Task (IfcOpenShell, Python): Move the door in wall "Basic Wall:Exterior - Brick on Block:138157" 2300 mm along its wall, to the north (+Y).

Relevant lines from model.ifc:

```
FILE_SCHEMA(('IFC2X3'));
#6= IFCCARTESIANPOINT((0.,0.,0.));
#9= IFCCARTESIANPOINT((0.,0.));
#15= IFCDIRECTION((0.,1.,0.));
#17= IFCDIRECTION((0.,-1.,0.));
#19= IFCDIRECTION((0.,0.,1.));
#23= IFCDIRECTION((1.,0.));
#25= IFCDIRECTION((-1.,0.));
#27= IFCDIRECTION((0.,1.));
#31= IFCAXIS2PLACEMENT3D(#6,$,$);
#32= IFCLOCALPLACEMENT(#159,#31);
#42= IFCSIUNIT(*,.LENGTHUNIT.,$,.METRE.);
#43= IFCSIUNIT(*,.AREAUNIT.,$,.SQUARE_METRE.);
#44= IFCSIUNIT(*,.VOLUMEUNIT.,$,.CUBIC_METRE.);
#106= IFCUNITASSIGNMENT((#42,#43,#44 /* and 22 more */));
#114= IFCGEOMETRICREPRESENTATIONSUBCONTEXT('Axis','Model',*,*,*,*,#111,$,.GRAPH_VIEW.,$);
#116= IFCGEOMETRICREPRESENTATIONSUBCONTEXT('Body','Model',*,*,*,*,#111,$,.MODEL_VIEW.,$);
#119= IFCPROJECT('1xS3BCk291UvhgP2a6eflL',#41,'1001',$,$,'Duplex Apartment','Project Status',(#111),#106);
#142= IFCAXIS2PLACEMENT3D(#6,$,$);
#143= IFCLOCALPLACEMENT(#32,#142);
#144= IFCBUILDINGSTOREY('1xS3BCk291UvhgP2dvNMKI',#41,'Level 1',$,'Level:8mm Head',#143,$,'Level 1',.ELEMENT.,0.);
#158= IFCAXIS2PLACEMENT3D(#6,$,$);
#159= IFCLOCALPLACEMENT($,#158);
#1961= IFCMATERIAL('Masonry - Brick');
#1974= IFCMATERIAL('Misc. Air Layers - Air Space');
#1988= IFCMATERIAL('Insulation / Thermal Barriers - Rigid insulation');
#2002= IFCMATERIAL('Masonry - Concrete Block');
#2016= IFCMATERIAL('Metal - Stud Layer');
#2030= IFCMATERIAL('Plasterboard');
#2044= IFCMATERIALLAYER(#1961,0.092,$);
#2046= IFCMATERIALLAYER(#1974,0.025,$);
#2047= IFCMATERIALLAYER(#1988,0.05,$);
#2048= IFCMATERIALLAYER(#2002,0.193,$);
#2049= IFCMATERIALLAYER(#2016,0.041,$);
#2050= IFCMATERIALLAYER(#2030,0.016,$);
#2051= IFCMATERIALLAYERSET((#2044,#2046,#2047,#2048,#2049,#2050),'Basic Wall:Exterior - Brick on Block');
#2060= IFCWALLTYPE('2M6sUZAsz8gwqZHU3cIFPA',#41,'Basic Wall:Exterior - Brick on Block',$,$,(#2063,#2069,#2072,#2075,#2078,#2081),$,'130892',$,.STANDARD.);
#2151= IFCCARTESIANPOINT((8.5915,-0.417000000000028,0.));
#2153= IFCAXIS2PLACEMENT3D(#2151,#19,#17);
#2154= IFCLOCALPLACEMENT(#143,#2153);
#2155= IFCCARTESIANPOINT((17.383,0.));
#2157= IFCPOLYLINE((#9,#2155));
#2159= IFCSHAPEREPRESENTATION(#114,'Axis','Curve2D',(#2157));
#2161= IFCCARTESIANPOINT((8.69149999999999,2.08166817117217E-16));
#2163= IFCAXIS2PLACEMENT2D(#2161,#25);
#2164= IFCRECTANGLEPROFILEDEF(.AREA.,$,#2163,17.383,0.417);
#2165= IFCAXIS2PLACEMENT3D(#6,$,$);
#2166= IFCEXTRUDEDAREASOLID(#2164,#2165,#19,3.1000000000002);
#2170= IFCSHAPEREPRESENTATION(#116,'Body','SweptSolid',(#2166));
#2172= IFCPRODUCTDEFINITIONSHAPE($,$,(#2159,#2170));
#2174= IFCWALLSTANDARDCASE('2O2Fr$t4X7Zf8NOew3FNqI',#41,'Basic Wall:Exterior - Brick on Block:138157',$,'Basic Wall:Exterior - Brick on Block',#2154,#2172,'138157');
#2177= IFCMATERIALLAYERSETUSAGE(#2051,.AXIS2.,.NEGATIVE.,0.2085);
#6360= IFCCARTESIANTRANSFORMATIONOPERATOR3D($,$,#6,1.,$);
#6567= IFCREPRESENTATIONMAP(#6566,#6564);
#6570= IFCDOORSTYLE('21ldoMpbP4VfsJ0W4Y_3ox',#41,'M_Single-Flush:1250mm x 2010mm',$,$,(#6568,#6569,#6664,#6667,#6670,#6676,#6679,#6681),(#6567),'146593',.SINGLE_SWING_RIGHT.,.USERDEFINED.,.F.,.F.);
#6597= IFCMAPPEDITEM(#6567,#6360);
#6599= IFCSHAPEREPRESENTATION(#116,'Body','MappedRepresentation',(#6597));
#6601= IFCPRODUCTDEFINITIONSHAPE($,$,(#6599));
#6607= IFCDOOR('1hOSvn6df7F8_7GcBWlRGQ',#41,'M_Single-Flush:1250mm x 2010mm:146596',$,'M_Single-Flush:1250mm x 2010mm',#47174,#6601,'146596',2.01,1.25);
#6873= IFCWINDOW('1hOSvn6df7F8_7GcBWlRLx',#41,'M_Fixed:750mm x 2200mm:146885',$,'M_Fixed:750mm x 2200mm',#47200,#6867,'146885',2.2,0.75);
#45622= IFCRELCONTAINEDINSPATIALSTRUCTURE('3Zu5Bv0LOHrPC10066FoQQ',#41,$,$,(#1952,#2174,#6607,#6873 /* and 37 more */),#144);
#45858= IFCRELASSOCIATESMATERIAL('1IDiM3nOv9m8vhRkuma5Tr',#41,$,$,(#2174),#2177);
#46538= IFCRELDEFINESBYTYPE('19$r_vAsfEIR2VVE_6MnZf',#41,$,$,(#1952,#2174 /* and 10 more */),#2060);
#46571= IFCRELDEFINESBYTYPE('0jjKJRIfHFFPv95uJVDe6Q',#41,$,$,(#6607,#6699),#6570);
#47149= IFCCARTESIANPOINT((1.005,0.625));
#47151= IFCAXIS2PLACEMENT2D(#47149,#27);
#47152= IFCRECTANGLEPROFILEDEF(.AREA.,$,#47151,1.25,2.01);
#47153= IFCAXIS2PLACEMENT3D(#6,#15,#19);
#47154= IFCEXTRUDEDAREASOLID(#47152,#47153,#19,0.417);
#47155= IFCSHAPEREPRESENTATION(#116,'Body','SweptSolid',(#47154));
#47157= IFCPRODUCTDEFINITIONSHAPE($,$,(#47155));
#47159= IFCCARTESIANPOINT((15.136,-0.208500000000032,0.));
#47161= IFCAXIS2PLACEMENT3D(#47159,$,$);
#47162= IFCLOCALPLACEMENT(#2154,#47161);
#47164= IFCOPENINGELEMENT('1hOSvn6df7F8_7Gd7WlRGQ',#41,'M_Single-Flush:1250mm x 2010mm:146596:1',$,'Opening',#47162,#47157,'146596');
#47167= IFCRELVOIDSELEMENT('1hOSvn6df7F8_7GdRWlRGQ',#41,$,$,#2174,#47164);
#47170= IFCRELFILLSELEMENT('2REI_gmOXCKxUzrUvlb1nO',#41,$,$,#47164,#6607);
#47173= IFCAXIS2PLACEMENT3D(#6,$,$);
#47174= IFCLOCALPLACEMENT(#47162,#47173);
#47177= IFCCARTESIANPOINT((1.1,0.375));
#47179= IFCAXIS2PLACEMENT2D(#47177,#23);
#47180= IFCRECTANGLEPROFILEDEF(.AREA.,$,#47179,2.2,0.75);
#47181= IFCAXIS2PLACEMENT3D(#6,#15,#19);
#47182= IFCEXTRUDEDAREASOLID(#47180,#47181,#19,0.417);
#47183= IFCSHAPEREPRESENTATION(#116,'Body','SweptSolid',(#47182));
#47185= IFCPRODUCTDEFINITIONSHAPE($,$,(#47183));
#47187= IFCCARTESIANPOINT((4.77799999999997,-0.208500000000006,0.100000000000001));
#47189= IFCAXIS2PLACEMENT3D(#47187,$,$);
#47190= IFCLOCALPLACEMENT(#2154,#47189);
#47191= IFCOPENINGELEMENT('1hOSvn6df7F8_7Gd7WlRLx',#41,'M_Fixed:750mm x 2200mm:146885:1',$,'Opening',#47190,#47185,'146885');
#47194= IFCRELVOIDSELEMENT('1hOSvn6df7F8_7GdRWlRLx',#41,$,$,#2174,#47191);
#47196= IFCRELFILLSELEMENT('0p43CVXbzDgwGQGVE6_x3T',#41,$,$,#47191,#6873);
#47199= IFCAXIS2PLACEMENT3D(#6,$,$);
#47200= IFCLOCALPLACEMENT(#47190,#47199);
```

```python
import ifcopenshell
import ifcopenshell.api.geometry
import ifcopenshell.util.placement
import ifcopenshell.util.unit

model = ifcopenshell.open("model.ifc")
unit_scale = ifcopenshell.util.unit.calculate_unit_scale(model)

door = model.by_id(6607)
opening = door.FillsVoids[0].RelatingOpeningElement
wall = opening.VoidsElements[0].RelatingBuildingElement

wall_matrix = ifcopenshell.util.placement.get_local_placement(wall.ObjectPlacement)
shift = wall_matrix[:3, 0] * -2.3 / unit_scale
before = ifcopenshell.util.placement.get_local_placement(door.ObjectPlacement)[:3, 3].copy()

# The door is placed relative to its opening, so it follows when the opening moves.
matrix = ifcopenshell.util.placement.get_local_placement(opening.ObjectPlacement)
matrix[:3, 3] += shift
ifcopenshell.api.geometry.edit_object_placement(
    model, product=opening, matrix=matrix, is_si=False, should_transform_children=True
)

after = ifcopenshell.util.placement.get_local_placement(door.ObjectPlacement)[:3, 3]
print("door moved by", (after - before).round(3) + 0.0)

model.write("model-out.ifc")
```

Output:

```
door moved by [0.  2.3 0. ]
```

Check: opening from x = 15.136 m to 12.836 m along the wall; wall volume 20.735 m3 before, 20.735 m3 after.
